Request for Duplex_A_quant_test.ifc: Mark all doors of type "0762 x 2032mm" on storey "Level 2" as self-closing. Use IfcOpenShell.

First a look at what the model holds.

```python
import ifcopenshell
import ifcopenshell.util.element

model = ifcopenshell.open("Duplex_A_quant_test.ifc")
print(model.schema)
storey = next(s for s in model.by_type("IfcBuildingStorey") if s.Name == "Level 2")
doors = [e for e in ifcopenshell.util.element.get_decomposition(storey) if e.is_a("IfcDoor")]
seen = {}
for e in doors:
    element_type = ifcopenshell.util.element.get_type(e)
    key = (element_type.Name if element_type != e and element_type else None, ifcopenshell.util.element.get_pset(e, "Pset_DoorCommon", "SelfClosing"))
    seen[key] = seen.get(key, 0) + 1
for (name, value), count in sorted(seen.items(), key=str):
    print(count, "x", name, "|", value)
```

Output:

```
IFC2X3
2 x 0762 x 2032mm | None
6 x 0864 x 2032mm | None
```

```python
import ifcopenshell
import ifcopenshell.api.pset
import ifcopenshell.util.element

model = ifcopenshell.open("Duplex_A_quant_test.ifc")

storey = next(s for s in model.by_type("IfcBuildingStorey") if s.Name == "Level 2")
doors = [e for e in ifcopenshell.util.element.get_decomposition(storey) if e.is_a("IfcDoor")]

count = 0
for e in doors:
    element_type = ifcopenshell.util.element.get_type(e)
    if element_type in (None, e) or element_type.Name != "0762 x 2032mm":
        continue
    # add_pset returns the element's existing set when there is one.
    pset = ifcopenshell.api.pset.add_pset(model, product=e, name="Pset_DoorCommon")
    ifcopenshell.api.pset.edit_pset(model, pset=pset, properties={"SelfClosing": True})
    count += 1

print(count, "doors updated")

model.write("Duplex_A_quant_test_rev.ifc")
```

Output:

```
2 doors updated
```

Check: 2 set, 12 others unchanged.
